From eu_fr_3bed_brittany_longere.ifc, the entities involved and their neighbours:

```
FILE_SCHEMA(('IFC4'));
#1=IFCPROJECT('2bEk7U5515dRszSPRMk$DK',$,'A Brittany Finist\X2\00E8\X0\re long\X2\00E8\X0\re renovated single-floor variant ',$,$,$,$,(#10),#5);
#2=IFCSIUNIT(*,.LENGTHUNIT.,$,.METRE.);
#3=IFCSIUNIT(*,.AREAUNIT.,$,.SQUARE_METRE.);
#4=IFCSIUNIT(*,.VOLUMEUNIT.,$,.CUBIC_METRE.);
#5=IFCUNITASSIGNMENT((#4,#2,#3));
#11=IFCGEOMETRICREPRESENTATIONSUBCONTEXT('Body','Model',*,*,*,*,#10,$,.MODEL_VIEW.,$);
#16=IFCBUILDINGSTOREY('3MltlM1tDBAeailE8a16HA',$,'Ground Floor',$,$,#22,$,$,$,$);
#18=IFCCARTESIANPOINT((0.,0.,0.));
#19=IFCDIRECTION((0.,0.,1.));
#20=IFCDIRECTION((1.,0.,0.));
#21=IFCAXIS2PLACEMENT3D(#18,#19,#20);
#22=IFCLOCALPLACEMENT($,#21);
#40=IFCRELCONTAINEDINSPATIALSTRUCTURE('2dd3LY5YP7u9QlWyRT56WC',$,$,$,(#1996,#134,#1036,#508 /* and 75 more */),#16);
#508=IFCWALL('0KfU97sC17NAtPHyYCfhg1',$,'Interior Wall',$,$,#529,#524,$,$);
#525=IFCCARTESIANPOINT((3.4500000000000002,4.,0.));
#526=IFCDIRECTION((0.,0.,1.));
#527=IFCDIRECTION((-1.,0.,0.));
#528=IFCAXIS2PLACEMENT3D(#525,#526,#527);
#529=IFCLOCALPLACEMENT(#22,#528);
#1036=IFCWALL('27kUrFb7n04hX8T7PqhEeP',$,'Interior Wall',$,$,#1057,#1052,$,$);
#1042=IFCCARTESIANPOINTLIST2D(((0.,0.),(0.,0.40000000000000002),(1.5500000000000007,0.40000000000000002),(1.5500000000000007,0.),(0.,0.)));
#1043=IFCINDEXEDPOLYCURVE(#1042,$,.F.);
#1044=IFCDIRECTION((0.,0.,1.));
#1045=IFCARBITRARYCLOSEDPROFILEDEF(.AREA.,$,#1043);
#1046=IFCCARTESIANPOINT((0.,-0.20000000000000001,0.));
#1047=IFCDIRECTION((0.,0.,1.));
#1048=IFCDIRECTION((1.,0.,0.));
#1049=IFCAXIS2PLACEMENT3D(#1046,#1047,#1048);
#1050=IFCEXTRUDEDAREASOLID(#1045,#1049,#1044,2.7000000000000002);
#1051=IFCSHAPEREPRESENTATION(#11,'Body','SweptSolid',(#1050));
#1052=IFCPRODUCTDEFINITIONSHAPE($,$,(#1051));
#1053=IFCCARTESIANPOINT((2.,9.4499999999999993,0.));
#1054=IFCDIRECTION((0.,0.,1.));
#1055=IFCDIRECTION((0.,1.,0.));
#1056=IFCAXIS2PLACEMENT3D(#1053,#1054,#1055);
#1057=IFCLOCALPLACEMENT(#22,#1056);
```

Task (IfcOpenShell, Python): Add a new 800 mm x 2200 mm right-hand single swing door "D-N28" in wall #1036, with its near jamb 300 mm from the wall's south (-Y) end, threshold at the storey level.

```python
import numpy as np
import ifcopenshell
import ifcopenshell.api.feature
import ifcopenshell.api.geometry
import ifcopenshell.api.root
import ifcopenshell.api.spatial
import ifcopenshell.geom
import ifcopenshell.util.element
import ifcopenshell.util.placement
import ifcopenshell.util.representation
import ifcopenshell.util.shape
import ifcopenshell.util.unit

model = ifcopenshell.open("eu_fr_3bed_brittany_longere.ifc")
unit_scale = ifcopenshell.util.unit.calculate_unit_scale(model)
settings = ifcopenshell.geom.settings()


def volume(element):
    """Net volume in cubic metres, openings subtracted."""
    shape = ifcopenshell.geom.create_shape(settings, element)
    return ifcopenshell.util.shape.get_volume(shape.geometry)


wall = model.by_guid("27kUrFb7n04hX8T7PqhEeP")
storey = ifcopenshell.util.element.get_container(wall, ifc_class="IfcBuildingStorey")
context = ifcopenshell.util.representation.get_context(model, "Model", "Body", "MODEL_VIEW")
before = volume(wall)

width, height, from_end, sill = 0.8, 2.2, 0.3, 0.0  # metres

# The wall runs along its own X axis, and the end named is its -X end.
wall_shape = ifcopenshell.geom.create_shape(settings, wall)
x, y, z = ifcopenshell.util.shape.get_vertices(wall_shape.geometry).T
start = x.min() + from_end
face, thickness = float(y.min()), float(y.max() - y.min())
wall_matrix = ifcopenshell.util.placement.get_local_placement(wall.ObjectPlacement)
level = ifcopenshell.util.placement.get_local_placement(storey.ObjectPlacement)[2, 3]


def in_wall(x, y):
    """Placement at x, y metres in the wall's axes, at sill height."""
    matrix = wall_matrix.copy()
    matrix[:, 3] = wall_matrix @ np.array([x / unit_scale, y / unit_scale, 0.0, 1.0])
    matrix[2, 3] = level + sill / unit_scale
    return matrix


# Opening: a box that overshoots both wall faces by 50 mm.
opening = ifcopenshell.api.root.create_entity(model, ifc_class="IfcOpeningElement", predefined_type="OPENING")
box = ifcopenshell.api.geometry.add_wall_representation(
    model, context=context, length=width, height=height, thickness=thickness + 0.1
)
ifcopenshell.api.geometry.assign_representation(model, product=opening, representation=box)
ifcopenshell.api.geometry.edit_object_placement(model, product=opening, matrix=in_wall(start, face - 0.05), is_si=False)
ifcopenshell.api.feature.add_feature(model, feature=opening, element=wall)

door = ifcopenshell.api.root.create_entity(model, ifc_class="IfcDoor", name="D-N28", predefined_type="DOOR")
door.OverallWidth, door.OverallHeight = width / unit_scale, height / unit_scale
door.OperationType = "SINGLE_SWING_RIGHT"
body = ifcopenshell.api.geometry.add_door_representation(
    model,
    context=context,
    overall_width=door.OverallWidth,
    overall_height=door.OverallHeight,
    operation_type="SINGLE_SWING_RIGHT",
    lining_properties={"LiningDepth": thickness / unit_scale, "ThresholdDepth": thickness / unit_scale},
)
ifcopenshell.api.geometry.assign_representation(model, product=door, representation=body)
ifcopenshell.api.spatial.assign_container(model, products=[door], relating_structure=storey)
ifcopenshell.api.feature.add_filling(model, opening=opening, element=door)

# The lining spans the wall, so the door starts at the wall face.
ifcopenshell.api.geometry.edit_object_placement(model, product=door, matrix=in_wall(start, face), is_si=False)

after = volume(wall)

print(f"wall volume {before:.3f} -> {after:.3f} m3")

model.write("eu_fr_3bed_brittany_longere_v2.ifc")
```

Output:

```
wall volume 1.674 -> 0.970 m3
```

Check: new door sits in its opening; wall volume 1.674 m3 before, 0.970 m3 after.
